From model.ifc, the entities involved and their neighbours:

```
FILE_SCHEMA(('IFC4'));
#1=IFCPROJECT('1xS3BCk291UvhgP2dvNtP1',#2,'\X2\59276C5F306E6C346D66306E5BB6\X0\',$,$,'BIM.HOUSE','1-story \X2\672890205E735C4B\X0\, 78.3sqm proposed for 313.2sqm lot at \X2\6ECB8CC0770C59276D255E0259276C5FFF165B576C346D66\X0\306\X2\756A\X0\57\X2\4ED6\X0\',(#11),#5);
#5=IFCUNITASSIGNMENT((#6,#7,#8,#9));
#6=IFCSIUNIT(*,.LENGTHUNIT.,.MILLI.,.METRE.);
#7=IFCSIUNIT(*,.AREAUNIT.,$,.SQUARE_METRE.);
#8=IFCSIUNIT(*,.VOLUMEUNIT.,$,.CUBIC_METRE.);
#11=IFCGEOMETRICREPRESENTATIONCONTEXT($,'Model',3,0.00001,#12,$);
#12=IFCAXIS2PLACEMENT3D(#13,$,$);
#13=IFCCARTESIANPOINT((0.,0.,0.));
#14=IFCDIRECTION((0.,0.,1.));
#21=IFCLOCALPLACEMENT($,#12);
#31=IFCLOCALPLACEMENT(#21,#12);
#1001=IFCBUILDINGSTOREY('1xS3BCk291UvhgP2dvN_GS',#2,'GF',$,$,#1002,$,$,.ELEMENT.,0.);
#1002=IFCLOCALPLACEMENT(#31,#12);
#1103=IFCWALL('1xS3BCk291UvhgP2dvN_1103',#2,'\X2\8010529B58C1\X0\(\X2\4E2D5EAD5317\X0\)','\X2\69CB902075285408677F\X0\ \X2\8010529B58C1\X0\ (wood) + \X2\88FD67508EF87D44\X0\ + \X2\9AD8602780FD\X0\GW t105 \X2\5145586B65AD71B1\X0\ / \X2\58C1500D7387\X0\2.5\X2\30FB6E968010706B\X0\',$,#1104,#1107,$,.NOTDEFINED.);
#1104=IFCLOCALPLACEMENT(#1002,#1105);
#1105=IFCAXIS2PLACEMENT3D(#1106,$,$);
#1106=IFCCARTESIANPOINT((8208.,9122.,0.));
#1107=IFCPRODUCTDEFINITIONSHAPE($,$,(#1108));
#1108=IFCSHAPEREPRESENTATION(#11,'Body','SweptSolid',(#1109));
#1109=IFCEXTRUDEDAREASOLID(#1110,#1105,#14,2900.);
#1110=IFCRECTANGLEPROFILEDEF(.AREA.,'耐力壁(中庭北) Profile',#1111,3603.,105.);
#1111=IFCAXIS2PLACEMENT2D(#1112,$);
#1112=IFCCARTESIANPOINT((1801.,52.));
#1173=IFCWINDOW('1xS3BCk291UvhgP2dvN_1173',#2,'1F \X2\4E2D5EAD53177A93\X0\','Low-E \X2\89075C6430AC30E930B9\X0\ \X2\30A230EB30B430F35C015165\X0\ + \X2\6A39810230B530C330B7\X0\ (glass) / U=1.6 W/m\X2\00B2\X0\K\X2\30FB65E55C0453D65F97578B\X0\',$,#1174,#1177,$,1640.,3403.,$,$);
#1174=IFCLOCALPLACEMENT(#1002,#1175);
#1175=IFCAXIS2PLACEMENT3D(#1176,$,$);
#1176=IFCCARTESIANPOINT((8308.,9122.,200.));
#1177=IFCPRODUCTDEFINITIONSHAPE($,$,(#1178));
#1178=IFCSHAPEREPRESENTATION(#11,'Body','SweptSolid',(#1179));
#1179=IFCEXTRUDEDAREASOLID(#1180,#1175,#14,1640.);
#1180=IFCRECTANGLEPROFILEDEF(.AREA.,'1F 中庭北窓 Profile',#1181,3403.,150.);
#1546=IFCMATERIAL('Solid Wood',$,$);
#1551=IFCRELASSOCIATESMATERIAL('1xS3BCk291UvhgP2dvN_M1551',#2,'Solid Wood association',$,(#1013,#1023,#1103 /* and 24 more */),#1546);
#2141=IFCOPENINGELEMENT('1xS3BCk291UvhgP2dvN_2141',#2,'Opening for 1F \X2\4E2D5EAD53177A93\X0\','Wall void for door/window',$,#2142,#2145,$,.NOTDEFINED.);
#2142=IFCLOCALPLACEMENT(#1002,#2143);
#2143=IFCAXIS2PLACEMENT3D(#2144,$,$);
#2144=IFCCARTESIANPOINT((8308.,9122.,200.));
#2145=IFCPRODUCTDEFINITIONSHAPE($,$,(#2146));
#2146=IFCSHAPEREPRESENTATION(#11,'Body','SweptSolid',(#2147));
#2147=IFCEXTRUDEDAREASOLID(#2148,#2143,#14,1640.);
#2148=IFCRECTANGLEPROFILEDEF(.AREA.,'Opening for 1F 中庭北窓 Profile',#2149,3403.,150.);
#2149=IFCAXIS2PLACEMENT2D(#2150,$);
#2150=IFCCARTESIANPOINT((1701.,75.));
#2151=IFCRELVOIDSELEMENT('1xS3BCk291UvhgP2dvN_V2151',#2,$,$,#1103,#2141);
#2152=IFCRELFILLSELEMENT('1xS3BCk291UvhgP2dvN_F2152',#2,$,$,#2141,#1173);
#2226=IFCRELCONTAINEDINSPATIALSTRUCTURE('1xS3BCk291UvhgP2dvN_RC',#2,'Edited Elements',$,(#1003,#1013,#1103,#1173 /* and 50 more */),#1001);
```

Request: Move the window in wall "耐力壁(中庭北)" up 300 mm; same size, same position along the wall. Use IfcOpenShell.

```python
import numpy as np
import ifcopenshell
import ifcopenshell.api.geometry
import ifcopenshell.util.placement
import ifcopenshell.util.unit

model = ifcopenshell.open("model.ifc")
unit_scale = ifcopenshell.util.unit.calculate_unit_scale(model)

window = model.by_guid("1xS3BCk291UvhgP2dvN_1173")
opening = window.FillsVoids[0].RelatingOpeningElement
dz = 0.3 / unit_scale

shift = np.array([0.0, 0.0, dz])
# The window is not placed relative to its opening, so move both.
for product in (opening, window):
    matrix = ifcopenshell.util.placement.get_local_placement(product.ObjectPlacement)
    matrix[:3, 3] += shift
    ifcopenshell.api.geometry.edit_object_placement(model, product=product, matrix=matrix, is_si=False)

print(f"moved by {dz * unit_scale:+.3f} m")

model.write("model_rev.ifc")
```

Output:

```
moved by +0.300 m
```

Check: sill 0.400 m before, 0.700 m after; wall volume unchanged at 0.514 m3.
